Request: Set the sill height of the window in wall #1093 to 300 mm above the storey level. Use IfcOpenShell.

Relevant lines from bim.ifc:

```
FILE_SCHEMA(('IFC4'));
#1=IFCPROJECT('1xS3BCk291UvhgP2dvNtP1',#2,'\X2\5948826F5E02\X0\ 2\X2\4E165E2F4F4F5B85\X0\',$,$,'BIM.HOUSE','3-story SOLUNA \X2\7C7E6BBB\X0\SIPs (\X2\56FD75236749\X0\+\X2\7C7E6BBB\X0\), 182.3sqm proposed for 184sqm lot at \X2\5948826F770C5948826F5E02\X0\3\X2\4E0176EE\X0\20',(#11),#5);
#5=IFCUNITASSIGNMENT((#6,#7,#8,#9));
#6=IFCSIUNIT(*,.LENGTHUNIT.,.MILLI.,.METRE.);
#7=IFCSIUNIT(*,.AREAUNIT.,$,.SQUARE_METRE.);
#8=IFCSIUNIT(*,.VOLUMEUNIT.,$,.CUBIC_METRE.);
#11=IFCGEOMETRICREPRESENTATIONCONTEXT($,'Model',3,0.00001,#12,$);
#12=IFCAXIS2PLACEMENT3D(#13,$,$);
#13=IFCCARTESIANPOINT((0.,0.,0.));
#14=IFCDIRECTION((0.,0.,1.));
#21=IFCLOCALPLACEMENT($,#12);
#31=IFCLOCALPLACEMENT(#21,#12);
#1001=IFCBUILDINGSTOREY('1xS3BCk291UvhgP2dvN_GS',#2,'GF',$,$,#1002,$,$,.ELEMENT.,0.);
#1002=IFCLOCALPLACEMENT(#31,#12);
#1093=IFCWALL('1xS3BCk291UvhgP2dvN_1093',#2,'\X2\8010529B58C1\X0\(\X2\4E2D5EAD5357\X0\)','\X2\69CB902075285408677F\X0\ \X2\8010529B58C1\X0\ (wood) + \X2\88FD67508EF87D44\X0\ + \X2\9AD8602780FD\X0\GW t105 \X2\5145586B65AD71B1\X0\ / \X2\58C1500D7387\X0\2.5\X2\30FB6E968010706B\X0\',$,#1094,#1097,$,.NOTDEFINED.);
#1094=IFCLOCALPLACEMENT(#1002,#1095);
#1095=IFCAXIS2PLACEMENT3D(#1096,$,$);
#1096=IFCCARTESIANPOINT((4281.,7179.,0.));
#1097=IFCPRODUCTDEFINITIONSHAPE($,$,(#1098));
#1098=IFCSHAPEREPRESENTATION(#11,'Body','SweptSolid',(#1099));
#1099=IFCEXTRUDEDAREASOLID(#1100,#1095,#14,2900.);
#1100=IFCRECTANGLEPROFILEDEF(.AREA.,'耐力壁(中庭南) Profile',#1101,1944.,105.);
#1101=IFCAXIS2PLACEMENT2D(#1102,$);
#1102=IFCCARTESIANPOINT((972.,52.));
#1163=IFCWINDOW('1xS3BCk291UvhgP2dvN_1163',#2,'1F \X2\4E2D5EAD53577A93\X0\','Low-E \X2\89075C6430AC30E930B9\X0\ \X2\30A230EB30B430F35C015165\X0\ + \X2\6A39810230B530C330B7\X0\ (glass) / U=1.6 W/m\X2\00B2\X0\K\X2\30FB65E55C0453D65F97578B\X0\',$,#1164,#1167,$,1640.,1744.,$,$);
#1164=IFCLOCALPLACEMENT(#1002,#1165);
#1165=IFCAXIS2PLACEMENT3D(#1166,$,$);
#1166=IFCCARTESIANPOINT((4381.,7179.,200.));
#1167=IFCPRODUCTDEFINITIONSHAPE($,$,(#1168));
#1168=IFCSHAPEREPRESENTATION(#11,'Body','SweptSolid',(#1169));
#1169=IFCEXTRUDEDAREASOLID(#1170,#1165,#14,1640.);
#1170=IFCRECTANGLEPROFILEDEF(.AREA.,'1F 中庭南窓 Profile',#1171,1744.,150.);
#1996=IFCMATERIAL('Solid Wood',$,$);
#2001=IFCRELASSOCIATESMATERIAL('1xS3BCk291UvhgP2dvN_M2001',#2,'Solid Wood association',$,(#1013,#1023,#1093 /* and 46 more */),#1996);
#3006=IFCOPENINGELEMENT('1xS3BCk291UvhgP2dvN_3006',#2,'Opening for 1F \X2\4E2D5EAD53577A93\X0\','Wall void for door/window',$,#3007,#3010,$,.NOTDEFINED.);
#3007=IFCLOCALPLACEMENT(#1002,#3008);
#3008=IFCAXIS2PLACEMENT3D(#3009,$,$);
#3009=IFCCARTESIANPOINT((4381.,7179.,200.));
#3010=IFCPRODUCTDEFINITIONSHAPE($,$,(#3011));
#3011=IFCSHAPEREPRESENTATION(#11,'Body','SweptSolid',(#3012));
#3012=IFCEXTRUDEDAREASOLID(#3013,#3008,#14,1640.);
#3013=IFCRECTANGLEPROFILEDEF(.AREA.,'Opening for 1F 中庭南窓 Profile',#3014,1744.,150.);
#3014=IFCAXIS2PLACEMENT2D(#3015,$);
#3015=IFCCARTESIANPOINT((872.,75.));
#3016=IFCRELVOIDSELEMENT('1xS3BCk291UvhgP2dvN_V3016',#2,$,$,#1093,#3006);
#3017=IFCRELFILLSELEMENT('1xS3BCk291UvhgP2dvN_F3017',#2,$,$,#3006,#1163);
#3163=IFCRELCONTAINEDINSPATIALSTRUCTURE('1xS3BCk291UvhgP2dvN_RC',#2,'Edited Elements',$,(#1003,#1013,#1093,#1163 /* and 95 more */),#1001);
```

```python
import numpy as np
import ifcopenshell
import ifcopenshell.api.geometry
import ifcopenshell.geom
import ifcopenshell.util.element
import ifcopenshell.util.placement
import ifcopenshell.util.shape
import ifcopenshell.util.unit

model = ifcopenshell.open("bim.ifc")
unit_scale = ifcopenshell.util.unit.calculate_unit_scale(model)

window = model.by_id(1163)
opening = window.FillsVoids[0].RelatingOpeningElement
storey = ifcopenshell.util.element.get_container(window, ifc_class="IfcBuildingStorey")
level = ifcopenshell.util.placement.get_local_placement(storey.ObjectPlacement)[2, 3]

# The opening's origin need not be at the sill, so measure its lowest point.
shape = ifcopenshell.geom.create_shape(ifcopenshell.geom.settings(), opening)
bottom = ifcopenshell.util.shape.get_shape_bottom_elevation(shape, shape.geometry) / unit_scale
dz = level + 0.3 / unit_scale - bottom

shift = np.array([0.0, 0.0, dz])
# The window is not placed relative to its opening, so move both.
for product in (opening, window):
    matrix = ifcopenshell.util.placement.get_local_placement(product.ObjectPlacement)
    matrix[:3, 3] += shift
    ifcopenshell.api.geometry.edit_object_placement(model, product=product, matrix=matrix, is_si=False)

print(f"moved by {dz * unit_scale:+.3f} m")

model.write("bim_updated.ifc")
```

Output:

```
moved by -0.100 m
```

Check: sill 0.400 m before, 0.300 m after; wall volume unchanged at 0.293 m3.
